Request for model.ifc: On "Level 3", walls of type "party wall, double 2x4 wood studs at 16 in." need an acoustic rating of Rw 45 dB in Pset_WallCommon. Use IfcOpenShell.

First a look at what the model holds.

```python
import ifcopenshell
import ifcopenshell.util.element

model = ifcopenshell.open("model.ifc")
print(model.schema)
storey = next(s for s in model.by_type("IfcBuildingStorey") if s.Name == "Level 3")
walls = [e for e in ifcopenshell.util.element.get_decomposition(storey) if e.is_a("IfcWall")]
seen = {}
for e in walls:
    element_type = ifcopenshell.util.element.get_type(e)
    key = (element_type.Name if element_type != e and element_type else None, ifcopenshell.util.element.get_pset(e, "Pset_WallCommon", "AcousticRating"))
    seen[key] = seen.get(key, 0) + 1
for (name, value), count in sorted(seen.items(), key=str):
    print(count, "x", name, "|", value)
```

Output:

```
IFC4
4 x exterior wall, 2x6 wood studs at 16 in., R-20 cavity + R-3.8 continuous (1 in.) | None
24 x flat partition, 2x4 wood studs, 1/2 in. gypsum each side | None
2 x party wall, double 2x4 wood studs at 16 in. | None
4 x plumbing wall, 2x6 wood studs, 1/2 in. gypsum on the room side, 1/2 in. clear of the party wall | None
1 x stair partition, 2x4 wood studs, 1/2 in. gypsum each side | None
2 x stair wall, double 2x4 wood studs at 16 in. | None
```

```python
import ifcopenshell
import ifcopenshell.api.pset
import ifcopenshell.util.element

model = ifcopenshell.open("model.ifc")

storey = next(s for s in model.by_type("IfcBuildingStorey") if s.Name == "Level 3")
walls = [e for e in ifcopenshell.util.element.get_decomposition(storey) if e.is_a("IfcWall")]

count = 0
for e in walls:
    element_type = ifcopenshell.util.element.get_type(e)
    if element_type in (None, e) or element_type.Name != "party wall, double 2x4 wood studs at 16 in.":
        continue
    # add_pset returns the element's existing set when there is one.
    pset = ifcopenshell.api.pset.add_pset(model, product=e, name="Pset_WallCommon")
    ifcopenshell.api.pset.edit_pset(model, pset=pset, properties={"AcousticRating": "Rw 45 dB"})
    count += 1

print(count, "walls updated")

model.write("model_v2.ifc")
```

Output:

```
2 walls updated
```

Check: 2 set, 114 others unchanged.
